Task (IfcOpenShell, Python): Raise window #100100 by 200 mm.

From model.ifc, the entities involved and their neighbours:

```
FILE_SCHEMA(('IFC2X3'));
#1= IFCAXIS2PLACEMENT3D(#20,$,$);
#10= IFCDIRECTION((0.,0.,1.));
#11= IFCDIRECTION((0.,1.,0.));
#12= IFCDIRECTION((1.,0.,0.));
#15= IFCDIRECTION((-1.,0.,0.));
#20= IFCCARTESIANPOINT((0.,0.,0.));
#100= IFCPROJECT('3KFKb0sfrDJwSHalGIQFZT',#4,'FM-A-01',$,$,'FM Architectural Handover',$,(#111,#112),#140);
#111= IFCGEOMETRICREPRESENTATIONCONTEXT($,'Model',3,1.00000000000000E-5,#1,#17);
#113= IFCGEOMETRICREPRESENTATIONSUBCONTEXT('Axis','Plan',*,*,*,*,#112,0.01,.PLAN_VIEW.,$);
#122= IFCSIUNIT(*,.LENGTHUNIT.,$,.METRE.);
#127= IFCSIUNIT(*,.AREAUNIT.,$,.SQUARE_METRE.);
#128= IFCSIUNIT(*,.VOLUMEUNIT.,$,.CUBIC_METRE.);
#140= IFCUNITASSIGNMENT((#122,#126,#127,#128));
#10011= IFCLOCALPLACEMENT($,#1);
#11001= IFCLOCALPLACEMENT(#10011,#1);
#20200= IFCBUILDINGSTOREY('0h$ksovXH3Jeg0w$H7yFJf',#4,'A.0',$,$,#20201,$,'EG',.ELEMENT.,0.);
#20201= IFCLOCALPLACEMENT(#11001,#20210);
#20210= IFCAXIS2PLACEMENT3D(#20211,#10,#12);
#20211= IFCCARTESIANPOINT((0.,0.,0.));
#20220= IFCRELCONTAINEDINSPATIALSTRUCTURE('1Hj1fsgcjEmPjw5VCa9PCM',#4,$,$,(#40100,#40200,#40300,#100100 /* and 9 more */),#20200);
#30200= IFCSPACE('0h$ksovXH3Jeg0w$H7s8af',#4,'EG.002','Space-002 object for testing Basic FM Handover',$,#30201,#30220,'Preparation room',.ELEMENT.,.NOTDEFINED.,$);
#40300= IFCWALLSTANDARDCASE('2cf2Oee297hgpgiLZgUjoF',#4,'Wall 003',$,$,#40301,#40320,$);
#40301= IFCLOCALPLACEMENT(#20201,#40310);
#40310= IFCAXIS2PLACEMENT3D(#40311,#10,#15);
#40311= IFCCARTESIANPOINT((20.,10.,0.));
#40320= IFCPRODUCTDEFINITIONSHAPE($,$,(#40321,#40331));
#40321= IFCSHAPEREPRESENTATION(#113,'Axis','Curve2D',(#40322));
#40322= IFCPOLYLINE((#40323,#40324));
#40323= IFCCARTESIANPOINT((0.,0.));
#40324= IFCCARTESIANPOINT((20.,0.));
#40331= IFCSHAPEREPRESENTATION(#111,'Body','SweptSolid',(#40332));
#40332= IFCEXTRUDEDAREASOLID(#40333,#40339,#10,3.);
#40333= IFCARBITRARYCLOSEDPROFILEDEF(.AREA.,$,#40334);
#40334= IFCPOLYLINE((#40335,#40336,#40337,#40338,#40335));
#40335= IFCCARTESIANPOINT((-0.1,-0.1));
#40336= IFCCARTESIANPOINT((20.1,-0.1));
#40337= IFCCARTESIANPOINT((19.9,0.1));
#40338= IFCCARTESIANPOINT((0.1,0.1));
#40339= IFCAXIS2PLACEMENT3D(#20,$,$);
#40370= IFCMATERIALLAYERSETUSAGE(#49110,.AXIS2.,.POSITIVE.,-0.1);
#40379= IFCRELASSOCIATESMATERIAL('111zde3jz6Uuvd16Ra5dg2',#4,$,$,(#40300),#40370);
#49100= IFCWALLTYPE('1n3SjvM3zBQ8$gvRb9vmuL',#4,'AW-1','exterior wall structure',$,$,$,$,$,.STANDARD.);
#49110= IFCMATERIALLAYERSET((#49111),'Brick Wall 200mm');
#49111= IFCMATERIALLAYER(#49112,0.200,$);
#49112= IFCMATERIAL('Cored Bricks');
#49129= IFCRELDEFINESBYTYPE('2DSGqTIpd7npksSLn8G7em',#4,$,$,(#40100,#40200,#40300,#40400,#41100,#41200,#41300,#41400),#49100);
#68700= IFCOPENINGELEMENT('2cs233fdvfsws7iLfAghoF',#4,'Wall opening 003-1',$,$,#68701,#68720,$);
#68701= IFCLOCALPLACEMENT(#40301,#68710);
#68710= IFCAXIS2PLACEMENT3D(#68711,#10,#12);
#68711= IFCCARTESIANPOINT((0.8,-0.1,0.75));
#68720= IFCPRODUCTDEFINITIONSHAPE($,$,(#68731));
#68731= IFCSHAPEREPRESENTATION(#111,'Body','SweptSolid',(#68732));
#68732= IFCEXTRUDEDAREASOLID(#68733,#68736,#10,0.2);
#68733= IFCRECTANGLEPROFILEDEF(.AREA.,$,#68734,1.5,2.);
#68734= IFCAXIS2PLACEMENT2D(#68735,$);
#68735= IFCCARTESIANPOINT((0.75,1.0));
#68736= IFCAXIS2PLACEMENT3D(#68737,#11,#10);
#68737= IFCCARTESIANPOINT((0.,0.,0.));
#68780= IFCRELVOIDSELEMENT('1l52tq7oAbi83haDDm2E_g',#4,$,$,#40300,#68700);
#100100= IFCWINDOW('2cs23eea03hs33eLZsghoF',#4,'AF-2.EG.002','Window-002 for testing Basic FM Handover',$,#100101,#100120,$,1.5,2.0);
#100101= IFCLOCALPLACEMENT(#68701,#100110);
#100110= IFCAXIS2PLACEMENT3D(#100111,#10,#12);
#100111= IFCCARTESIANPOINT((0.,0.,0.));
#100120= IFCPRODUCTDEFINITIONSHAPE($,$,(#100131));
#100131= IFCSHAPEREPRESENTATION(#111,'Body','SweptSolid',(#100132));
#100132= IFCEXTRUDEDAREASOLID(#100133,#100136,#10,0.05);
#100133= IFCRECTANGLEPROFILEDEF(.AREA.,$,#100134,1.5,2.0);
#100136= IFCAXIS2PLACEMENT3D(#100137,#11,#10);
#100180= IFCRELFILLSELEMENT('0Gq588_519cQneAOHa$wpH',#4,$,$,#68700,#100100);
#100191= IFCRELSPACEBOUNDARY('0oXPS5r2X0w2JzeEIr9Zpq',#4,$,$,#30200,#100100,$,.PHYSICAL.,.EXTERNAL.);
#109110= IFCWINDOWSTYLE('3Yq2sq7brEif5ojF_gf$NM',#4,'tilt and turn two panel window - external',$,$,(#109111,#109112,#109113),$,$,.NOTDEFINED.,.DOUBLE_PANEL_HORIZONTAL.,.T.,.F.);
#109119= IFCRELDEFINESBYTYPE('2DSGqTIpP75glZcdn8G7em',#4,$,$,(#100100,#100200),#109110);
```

```python
import numpy as np
import ifcopenshell
import ifcopenshell.api.geometry
import ifcopenshell.util.placement
import ifcopenshell.util.unit

model = ifcopenshell.open("model.ifc")
unit_scale = ifcopenshell.util.unit.calculate_unit_scale(model)

window = model.by_id(100100)
opening = window.FillsVoids[0].RelatingOpeningElement
dz = 0.2 / unit_scale

shift = np.array([0.0, 0.0, dz])
# The window is placed relative to its opening, so it follows when the opening moves.
matrix = ifcopenshell.util.placement.get_local_placement(opening.ObjectPlacement)
matrix[:3, 3] += shift
ifcopenshell.api.geometry.edit_object_placement(
    model, product=opening, matrix=matrix, is_si=False, should_transform_children=True
)

print(f"moved by {dz * unit_scale:+.3f} m")

model.write("model_edited.ifc")
```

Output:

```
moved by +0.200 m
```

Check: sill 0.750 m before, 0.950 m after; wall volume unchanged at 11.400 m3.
